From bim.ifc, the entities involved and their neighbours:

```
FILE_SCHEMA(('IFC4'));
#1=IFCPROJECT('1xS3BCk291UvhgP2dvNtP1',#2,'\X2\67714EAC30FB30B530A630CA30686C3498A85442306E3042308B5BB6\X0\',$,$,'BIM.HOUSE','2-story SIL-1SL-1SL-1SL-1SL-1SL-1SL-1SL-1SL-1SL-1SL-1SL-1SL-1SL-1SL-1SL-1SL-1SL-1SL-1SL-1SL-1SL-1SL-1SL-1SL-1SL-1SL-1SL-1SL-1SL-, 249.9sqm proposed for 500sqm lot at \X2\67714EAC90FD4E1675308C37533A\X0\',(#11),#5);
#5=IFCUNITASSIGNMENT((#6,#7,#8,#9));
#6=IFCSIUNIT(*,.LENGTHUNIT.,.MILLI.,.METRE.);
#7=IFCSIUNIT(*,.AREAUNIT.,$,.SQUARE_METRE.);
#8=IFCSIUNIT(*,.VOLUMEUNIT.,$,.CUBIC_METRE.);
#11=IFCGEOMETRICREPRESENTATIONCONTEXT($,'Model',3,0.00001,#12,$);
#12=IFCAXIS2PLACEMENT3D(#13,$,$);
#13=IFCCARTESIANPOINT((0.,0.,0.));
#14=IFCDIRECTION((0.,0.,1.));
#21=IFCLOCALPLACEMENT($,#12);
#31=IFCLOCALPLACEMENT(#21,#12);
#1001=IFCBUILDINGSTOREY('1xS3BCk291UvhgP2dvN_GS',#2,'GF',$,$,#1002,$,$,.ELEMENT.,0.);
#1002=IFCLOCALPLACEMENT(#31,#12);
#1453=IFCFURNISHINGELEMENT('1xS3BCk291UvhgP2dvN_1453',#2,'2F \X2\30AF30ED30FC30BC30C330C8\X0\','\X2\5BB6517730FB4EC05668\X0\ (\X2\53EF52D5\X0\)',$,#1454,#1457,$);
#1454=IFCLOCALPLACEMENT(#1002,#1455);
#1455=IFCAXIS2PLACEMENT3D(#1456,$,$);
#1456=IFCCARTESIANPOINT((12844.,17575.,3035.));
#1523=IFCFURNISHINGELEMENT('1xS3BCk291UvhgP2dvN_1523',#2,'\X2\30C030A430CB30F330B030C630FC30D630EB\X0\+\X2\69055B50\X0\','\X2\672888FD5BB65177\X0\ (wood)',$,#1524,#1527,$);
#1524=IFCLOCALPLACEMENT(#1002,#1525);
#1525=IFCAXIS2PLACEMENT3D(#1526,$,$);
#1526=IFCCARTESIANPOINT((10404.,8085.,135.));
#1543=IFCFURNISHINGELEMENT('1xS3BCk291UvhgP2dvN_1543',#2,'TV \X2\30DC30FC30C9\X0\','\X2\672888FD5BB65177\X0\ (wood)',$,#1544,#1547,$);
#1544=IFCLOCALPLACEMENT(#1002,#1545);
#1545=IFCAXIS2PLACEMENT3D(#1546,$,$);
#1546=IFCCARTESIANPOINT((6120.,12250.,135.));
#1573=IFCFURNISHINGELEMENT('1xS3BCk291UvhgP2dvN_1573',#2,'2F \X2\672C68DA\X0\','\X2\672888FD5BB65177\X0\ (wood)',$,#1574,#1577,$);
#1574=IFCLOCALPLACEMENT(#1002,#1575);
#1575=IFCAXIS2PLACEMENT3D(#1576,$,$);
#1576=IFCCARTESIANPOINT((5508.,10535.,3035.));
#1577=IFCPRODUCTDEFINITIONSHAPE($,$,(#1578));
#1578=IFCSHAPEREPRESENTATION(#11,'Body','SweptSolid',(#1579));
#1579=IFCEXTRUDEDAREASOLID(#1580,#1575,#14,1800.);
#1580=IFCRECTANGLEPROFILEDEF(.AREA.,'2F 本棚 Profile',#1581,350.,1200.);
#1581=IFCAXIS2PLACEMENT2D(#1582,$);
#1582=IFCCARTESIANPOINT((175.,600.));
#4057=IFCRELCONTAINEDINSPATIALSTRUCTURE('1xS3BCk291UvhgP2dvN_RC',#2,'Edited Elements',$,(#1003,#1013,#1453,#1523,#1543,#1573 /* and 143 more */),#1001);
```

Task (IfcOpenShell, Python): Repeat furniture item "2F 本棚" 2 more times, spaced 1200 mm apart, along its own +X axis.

```python
import ifcopenshell
import ifcopenshell.api.geometry
import ifcopenshell.api.root
import ifcopenshell.util.element
import ifcopenshell.util.placement

model = ifcopenshell.open("bim.ifc")


def reuse_history(source, copy):
    """copy_class also copies each property set's owner history, people and application; keep the originals."""
    for rel in copy.IsDefinedBy:
        if rel.is_a("IfcRelDefinesByProperties") and (history := rel.RelatingPropertyDefinition.OwnerHistory):
            rel.RelatingPropertyDefinition.OwnerHistory = source.OwnerHistory
            ifcopenshell.util.element.remove_deep2(model, history)


source = model.by_guid("1xS3BCk291UvhgP2dvN_1573")
base = ifcopenshell.util.placement.get_local_placement(source.ObjectPlacement)
step = base[:3, 0] * 1200.0

for i in range(1, 3):
    copy = ifcopenshell.api.root.copy_class(model, product=source)
    copy.Representation = ifcopenshell.util.element.copy_deep(
        model, source.Representation, exclude=["IfcGeometricRepresentationContext", "IfcRepresentationMap"]
    )
    reuse_history(source, copy)
    matrix = base.copy()
    matrix[:3, 3] += i * step
    print("added at", matrix[:3, 3].round(3) + 0.0)
    ifcopenshell.api.geometry.edit_object_placement(model, product=copy, matrix=matrix, is_si=False)

model.write("bim_rev.ifc")
```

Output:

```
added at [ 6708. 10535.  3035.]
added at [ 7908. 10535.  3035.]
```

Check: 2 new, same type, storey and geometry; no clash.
